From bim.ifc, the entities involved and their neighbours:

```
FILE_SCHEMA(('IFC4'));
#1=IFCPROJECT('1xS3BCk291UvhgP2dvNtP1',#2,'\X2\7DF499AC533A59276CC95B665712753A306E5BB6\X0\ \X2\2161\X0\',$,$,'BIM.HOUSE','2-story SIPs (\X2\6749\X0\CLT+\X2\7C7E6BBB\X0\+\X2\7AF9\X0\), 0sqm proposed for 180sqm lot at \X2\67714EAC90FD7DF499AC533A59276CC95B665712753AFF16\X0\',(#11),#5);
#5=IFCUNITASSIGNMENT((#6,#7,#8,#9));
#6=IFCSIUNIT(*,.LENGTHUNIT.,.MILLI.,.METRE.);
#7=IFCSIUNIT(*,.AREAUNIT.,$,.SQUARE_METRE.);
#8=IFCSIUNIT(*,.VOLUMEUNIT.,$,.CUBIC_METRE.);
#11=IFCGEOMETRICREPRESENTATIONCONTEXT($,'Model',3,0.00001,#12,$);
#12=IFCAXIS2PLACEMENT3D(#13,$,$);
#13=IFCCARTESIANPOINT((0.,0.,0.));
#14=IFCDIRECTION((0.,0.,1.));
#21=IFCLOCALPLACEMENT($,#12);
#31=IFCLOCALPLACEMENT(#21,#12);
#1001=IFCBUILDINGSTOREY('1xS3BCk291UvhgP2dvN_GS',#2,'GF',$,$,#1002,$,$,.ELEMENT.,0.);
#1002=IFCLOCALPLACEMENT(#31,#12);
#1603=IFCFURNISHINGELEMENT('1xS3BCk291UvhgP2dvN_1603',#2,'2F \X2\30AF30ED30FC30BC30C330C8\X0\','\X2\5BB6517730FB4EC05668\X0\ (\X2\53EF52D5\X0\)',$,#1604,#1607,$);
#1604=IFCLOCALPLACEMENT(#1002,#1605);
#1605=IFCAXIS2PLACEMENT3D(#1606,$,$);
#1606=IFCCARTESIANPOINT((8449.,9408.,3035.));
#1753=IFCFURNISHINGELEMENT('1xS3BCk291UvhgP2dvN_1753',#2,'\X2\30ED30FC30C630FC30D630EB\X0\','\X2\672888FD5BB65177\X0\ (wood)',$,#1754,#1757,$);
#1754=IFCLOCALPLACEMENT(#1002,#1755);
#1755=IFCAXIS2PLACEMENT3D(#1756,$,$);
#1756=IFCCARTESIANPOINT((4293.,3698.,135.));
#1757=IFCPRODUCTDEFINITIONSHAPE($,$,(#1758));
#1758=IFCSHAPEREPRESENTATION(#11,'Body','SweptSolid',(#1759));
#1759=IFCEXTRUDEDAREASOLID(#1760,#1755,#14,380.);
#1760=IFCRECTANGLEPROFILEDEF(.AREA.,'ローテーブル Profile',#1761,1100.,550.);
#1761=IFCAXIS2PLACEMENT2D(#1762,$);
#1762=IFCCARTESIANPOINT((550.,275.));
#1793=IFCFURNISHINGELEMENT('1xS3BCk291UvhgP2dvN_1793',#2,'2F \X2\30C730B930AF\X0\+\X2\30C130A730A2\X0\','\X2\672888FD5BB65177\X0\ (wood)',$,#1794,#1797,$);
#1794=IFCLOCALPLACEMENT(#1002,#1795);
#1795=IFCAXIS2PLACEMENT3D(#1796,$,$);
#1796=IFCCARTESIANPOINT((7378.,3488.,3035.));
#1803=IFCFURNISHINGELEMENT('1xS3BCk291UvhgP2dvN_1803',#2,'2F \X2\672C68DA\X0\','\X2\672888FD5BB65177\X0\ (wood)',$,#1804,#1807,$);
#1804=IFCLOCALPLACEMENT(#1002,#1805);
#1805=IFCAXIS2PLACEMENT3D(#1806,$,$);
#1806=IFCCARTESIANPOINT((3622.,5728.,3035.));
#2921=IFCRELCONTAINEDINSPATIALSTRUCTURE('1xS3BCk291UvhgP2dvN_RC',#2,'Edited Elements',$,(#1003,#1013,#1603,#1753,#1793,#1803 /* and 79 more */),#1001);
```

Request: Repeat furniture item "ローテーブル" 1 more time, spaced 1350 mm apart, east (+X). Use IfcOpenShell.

```python
import numpy as np
import ifcopenshell
import ifcopenshell.api.geometry
import ifcopenshell.api.root
import ifcopenshell.util.element
import ifcopenshell.util.placement
import ifcopenshell.util.unit

model = ifcopenshell.open("bim.ifc")
unit_scale = ifcopenshell.util.unit.calculate_unit_scale(model)


def reuse_history(source, copy):
    """copy_class also copies each property set's owner history, people and application; keep the originals."""
    for rel in copy.IsDefinedBy:
        if rel.is_a("IfcRelDefinesByProperties") and (history := rel.RelatingPropertyDefinition.OwnerHistory):
            rel.RelatingPropertyDefinition.OwnerHistory = source.OwnerHistory
            ifcopenshell.util.element.remove_deep2(model, history)


source = model.by_id(1753)
base = ifcopenshell.util.placement.get_local_placement(source.ObjectPlacement)
step = np.array([1.0, 0.0, 0.0]) * 1.35 / unit_scale

for i in range(1, 2):
    copy = ifcopenshell.api.root.copy_class(model, product=source)
    copy.Representation = ifcopenshell.util.element.copy_deep(
        model, source.Representation, exclude=["IfcGeometricRepresentationContext", "IfcRepresentationMap"]
    )
    reuse_history(source, copy)
    matrix = base.copy()
    matrix[:3, 3] += i * step
    print("added at", matrix[:3, 3].round(3) + 0.0)
    ifcopenshell.api.geometry.edit_object_placement(model, product=copy, matrix=matrix, is_si=False)

model.write("bim_v2.ifc")
```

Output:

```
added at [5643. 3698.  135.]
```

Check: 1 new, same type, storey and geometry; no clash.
